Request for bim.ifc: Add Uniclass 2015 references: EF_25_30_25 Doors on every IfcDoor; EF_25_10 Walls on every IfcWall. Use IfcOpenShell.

First a look at what the model holds.

```python
import ifcopenshell

model = ifcopenshell.open("bim.ifc")
print(model.schema)
print("classifications:", [c.Name for c in model.by_type("IfcClassification")])
for ifc_class in ("IfcDoor", "IfcRoof", "IfcStair", "IfcWall", "IfcWindow"):
    print(ifc_class, len(model.by_type(ifc_class)))
```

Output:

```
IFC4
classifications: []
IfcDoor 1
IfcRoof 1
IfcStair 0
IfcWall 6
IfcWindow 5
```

```python
import ifcopenshell
import ifcopenshell.api.classification

model = ifcopenshell.open("bim.ifc")

system = ifcopenshell.api.classification.add_classification(model, classification="Uniclass 2015")

codes = {
    "IfcDoor": ("EF_25_30_25", "Doors"),
    "IfcWall": ("EF_25_10", "Walls"),
}
for ifc_class, (code, name) in codes.items():
    products = model.by_type(ifc_class)
    ifcopenshell.api.classification.add_reference(
        model, products=products, classification=system, identification=code, name=name
    )
    print(code, len(products))

model.write("bim_updated.ifc")
```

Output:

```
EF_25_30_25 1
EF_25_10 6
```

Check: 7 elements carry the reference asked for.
